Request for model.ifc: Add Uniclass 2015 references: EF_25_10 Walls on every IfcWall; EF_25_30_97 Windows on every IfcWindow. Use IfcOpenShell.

First a look at what the model holds.

```python
import ifcopenshell

model = ifcopenshell.open("model.ifc")
print(model.schema)
print("classifications:", [c.Name for c in model.by_type("IfcClassification")])
for ifc_class in ("IfcDoor", "IfcRoof", "IfcStair", "IfcWall", "IfcWindow"):
    print(ifc_class, len(model.by_type(ifc_class)))
```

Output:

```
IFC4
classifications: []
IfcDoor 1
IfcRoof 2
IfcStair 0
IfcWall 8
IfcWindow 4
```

```python
import ifcopenshell
import ifcopenshell.api.classification

model = ifcopenshell.open("model.ifc")

system = ifcopenshell.api.classification.add_classification(model, classification="Uniclass 2015")

codes = {
    "IfcWall": ("EF_25_10", "Walls"),
    "IfcWindow": ("EF_25_30_97", "Windows"),
}
for ifc_class, (code, name) in codes.items():
    products = model.by_type(ifc_class)
    ifcopenshell.api.classification.add_reference(
        model, products=products, classification=system, identification=code, name=name
    )
    print(code, len(products))

model.write("model_v2.ifc")
```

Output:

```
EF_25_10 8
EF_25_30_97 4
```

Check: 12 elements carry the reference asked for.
